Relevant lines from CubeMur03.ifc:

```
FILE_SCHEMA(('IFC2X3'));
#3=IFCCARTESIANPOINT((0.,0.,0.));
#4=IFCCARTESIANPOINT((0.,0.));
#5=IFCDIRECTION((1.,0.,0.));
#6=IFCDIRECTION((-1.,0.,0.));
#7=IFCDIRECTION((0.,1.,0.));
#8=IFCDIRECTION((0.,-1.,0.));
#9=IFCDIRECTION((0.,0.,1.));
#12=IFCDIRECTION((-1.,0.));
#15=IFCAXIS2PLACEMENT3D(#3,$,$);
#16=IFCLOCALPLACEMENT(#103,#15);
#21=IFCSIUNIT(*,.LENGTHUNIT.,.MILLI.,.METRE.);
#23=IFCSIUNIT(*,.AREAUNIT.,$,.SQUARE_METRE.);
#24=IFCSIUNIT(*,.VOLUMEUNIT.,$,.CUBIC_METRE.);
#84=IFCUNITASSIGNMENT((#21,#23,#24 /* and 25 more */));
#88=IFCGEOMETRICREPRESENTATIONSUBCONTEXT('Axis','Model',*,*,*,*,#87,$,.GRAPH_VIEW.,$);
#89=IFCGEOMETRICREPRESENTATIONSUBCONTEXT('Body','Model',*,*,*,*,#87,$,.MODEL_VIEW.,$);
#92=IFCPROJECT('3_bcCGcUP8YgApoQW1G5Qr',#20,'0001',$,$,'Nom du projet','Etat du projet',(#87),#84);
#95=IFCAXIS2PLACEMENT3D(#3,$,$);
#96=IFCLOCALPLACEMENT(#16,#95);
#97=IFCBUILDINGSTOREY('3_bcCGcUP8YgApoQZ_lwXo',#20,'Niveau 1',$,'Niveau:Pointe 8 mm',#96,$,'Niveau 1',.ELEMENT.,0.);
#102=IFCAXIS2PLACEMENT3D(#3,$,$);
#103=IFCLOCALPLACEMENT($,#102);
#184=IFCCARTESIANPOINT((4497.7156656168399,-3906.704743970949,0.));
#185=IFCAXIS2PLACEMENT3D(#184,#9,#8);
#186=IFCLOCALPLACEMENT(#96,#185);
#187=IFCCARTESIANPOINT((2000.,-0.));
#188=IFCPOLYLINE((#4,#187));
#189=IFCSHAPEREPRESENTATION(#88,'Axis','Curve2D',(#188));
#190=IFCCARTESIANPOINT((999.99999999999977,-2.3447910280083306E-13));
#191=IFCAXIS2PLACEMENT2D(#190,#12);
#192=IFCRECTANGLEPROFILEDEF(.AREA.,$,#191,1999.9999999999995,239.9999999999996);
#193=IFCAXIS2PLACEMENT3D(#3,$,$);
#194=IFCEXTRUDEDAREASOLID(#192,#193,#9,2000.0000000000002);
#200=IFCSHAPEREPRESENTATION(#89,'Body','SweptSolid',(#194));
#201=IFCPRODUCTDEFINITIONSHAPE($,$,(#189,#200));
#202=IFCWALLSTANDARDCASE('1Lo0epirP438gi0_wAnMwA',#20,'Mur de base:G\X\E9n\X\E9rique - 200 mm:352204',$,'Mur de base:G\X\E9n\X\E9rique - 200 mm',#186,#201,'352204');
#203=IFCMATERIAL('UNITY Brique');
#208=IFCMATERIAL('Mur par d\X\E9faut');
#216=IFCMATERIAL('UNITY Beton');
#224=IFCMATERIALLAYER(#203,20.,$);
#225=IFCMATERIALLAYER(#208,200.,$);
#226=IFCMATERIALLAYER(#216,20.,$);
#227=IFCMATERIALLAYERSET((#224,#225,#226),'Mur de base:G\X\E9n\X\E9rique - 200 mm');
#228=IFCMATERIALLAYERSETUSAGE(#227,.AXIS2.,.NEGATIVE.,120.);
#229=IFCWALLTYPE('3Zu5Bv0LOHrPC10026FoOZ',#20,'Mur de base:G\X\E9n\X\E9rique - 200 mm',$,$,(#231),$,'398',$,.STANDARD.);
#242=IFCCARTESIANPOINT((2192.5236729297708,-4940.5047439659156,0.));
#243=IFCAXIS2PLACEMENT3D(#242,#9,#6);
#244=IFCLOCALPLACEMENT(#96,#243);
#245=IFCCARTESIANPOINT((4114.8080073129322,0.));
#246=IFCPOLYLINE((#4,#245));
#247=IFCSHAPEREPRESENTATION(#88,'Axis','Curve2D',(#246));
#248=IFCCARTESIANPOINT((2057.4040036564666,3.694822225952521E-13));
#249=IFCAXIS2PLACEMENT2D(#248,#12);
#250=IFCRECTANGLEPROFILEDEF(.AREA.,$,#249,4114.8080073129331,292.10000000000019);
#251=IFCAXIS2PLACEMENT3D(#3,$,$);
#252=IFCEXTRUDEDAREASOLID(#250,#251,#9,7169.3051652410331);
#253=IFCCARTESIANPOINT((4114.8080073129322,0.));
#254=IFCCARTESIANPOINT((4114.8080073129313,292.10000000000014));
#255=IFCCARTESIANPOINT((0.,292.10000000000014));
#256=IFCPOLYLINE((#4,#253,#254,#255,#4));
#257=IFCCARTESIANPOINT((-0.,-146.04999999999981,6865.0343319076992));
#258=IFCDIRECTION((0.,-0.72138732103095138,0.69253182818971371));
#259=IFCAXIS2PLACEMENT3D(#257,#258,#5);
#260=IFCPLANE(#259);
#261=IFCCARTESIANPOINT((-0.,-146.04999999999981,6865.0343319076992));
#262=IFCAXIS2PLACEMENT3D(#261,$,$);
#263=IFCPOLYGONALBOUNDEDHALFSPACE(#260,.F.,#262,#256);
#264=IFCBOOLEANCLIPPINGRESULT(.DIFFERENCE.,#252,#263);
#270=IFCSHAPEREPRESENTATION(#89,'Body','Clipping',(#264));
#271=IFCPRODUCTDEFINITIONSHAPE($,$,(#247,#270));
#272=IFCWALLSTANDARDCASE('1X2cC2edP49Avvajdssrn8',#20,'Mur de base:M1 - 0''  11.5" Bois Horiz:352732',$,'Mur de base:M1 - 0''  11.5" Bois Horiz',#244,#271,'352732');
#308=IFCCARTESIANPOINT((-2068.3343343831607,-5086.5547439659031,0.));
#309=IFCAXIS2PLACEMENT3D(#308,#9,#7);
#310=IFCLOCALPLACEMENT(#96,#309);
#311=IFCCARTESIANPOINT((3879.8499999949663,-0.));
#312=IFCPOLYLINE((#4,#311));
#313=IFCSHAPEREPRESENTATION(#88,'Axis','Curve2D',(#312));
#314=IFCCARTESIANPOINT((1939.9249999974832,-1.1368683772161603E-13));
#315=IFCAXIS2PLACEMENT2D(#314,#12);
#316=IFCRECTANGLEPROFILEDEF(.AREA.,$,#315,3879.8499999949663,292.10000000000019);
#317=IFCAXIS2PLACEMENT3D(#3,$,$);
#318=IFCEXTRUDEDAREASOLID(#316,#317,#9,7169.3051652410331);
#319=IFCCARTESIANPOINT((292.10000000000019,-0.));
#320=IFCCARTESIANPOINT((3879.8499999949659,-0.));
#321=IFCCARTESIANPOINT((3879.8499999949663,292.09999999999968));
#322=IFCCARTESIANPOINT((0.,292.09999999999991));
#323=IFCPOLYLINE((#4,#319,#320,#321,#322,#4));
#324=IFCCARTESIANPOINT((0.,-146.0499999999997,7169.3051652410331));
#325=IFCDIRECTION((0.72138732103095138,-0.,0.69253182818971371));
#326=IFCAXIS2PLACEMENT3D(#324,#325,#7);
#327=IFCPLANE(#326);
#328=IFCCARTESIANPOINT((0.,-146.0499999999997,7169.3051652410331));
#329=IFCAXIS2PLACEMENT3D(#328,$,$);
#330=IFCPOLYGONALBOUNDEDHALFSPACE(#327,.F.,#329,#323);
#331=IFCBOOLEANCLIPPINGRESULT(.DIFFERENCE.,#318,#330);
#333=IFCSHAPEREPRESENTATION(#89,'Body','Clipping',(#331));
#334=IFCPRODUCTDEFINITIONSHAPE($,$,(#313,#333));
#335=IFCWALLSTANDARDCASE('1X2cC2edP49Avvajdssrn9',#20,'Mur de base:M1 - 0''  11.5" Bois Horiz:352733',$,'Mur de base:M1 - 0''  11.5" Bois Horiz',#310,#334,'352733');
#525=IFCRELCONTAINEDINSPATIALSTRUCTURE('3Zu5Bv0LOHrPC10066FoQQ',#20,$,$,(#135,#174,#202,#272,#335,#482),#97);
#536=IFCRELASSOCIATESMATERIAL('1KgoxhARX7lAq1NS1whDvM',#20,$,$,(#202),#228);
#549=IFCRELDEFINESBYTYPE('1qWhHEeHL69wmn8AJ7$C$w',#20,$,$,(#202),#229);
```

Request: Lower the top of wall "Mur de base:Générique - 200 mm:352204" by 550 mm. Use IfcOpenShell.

```python
import ifcopenshell
import ifcopenshell.geom
import ifcopenshell.util.representation
import ifcopenshell.util.shape
import ifcopenshell.util.unit

model = ifcopenshell.open("CubeMur03.ifc")
unit_scale = ifcopenshell.util.unit.calculate_unit_scale(model)
settings = ifcopenshell.geom.settings()


def volume(element):
    """Net volume in cubic metres, openings subtracted."""
    shape = ifcopenshell.geom.create_shape(settings, element)
    return ifcopenshell.util.shape.get_volume(shape.geometry)


wall = model.by_guid("1Lo0epirP438gi0_wAnMwA")
before = volume(wall)

body = ifcopenshell.util.representation.get_representation(wall, "Model", "Body")
solid = body.Items[0]
old_height = solid.Depth
solid.Depth -= 0.55 / unit_scale
after = volume(wall)

print(f"height {old_height:g} -> {solid.Depth:g}, volume {before:.3f} -> {after:.3f} m3")

model.write("CubeMur03-out.ifc")
```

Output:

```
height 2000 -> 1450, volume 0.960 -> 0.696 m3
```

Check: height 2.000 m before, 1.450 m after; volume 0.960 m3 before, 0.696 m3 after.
